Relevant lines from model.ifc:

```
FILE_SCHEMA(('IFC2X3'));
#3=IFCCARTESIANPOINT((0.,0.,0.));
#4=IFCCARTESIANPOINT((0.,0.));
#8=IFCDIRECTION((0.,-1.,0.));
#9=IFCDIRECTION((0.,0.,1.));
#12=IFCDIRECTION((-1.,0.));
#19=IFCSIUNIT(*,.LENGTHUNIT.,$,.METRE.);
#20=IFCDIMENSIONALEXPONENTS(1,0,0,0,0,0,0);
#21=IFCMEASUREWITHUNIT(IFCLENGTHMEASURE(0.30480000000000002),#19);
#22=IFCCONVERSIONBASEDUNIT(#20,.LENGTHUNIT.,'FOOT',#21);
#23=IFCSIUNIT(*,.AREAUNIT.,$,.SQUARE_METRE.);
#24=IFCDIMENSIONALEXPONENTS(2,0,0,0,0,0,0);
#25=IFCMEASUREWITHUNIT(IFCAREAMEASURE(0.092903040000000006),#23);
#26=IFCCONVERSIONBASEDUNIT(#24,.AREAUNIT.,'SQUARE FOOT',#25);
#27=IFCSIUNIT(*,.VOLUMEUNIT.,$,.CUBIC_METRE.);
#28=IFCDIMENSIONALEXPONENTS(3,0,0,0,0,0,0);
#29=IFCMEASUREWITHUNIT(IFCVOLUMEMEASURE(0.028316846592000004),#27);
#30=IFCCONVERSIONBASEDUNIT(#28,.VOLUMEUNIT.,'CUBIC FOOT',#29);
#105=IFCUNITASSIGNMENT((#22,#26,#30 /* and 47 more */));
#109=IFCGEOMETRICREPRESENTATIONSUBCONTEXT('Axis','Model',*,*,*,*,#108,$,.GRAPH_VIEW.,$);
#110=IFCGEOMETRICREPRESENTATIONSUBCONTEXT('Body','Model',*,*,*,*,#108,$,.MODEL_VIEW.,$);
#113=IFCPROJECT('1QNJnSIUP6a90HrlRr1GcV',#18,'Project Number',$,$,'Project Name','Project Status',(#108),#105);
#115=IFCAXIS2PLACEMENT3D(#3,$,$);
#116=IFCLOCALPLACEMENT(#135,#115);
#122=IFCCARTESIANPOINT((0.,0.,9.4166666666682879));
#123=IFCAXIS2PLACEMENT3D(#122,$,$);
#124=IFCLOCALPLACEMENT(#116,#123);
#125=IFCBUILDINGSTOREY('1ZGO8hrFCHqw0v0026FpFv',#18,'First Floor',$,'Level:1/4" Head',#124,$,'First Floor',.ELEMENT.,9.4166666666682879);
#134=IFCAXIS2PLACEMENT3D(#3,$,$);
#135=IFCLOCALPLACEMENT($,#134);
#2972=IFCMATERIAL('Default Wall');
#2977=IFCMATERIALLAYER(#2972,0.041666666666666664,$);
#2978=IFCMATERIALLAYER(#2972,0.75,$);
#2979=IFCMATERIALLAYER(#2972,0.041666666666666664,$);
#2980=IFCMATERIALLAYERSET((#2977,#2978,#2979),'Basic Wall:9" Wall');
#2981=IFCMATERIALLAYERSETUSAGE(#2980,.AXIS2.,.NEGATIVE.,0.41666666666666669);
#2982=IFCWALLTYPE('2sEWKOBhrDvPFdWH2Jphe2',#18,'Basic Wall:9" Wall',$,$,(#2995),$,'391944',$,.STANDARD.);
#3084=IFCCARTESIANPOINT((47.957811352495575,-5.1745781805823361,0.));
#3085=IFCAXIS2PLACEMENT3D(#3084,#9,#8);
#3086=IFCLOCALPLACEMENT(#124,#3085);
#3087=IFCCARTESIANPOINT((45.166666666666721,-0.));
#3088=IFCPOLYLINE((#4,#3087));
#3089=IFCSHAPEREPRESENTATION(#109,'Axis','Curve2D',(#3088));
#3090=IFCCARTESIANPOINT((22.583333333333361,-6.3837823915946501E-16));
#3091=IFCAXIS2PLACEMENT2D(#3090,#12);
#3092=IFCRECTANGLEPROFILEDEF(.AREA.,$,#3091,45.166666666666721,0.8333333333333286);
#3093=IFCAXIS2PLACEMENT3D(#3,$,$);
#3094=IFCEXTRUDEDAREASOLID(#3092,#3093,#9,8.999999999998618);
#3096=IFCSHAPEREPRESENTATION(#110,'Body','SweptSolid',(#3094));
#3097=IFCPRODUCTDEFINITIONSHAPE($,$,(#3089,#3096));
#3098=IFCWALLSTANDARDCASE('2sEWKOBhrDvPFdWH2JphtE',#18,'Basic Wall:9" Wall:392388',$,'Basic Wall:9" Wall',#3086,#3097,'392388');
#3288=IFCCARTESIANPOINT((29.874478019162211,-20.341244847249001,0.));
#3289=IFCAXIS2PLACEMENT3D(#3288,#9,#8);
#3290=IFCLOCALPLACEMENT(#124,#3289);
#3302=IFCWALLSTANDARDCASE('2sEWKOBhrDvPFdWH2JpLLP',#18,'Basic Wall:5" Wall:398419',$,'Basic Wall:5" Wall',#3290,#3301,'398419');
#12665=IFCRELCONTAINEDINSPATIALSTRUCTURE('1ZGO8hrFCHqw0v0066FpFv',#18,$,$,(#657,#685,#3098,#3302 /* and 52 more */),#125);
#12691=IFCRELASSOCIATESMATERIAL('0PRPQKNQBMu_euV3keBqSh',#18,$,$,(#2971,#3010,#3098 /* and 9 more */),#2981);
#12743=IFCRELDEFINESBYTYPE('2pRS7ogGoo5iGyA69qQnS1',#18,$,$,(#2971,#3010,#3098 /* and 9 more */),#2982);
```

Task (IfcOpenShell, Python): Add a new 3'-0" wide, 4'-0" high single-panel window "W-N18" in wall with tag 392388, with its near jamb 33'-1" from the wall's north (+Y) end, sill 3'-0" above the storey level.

```python
import numpy as np
import ifcopenshell
import ifcopenshell.api.feature
import ifcopenshell.api.geometry
import ifcopenshell.api.root
import ifcopenshell.api.spatial
import ifcopenshell.api.type
import ifcopenshell.geom
import ifcopenshell.util.element
import ifcopenshell.util.placement
import ifcopenshell.util.representation
import ifcopenshell.util.shape
import ifcopenshell.util.unit

model = ifcopenshell.open("model.ifc")
unit_scale = ifcopenshell.util.unit.calculate_unit_scale(model)
settings = ifcopenshell.geom.settings()


def volume(element):
    """Net volume in cubic metres, openings subtracted."""
    shape = ifcopenshell.geom.create_shape(settings, element)
    return ifcopenshell.util.shape.get_volume(shape.geometry)


wall = model.by_guid("2sEWKOBhrDvPFdWH2JphtE")
storey = ifcopenshell.util.element.get_container(wall, ifc_class="IfcBuildingStorey")
context = ifcopenshell.util.representation.get_context(model, "Model", "Body", "MODEL_VIEW")
before = volume(wall)

width, height, from_end, sill = 0.9144, 1.2192, 10.0838, 0.9144  # metres

# The wall runs along its own X axis, and the end named is its -X end.
wall_shape = ifcopenshell.geom.create_shape(settings, wall)
x, y, z = ifcopenshell.util.shape.get_vertices(wall_shape.geometry).T
start = x.min() + from_end
face, thickness = float(y.min()), float(y.max() - y.min())
wall_matrix = ifcopenshell.util.placement.get_local_placement(wall.ObjectPlacement)
level = ifcopenshell.util.placement.get_local_placement(storey.ObjectPlacement)[2, 3]


def in_wall(x, y):
    """Placement at x, y metres in the wall's axes, at sill height."""
    matrix = wall_matrix.copy()
    matrix[:, 3] = wall_matrix @ np.array([x / unit_scale, y / unit_scale, 0.0, 1.0])
    matrix[2, 3] = level + sill / unit_scale
    return matrix


# Opening: a box that overshoots both wall faces by 50 mm.
opening = ifcopenshell.api.root.create_entity(model, ifc_class="IfcOpeningElement")
box = ifcopenshell.api.geometry.add_wall_representation(
    model, context=context, length=width, height=height, thickness=thickness + 0.1
)
ifcopenshell.api.geometry.assign_representation(model, product=opening, representation=box)
ifcopenshell.api.geometry.edit_object_placement(model, product=opening, matrix=in_wall(start, face - 0.05), is_si=False)
ifcopenshell.api.feature.add_feature(model, feature=opening, element=wall)

window = ifcopenshell.api.root.create_entity(model, ifc_class="IfcWindow", name="W-N18")
window.OverallWidth, window.OverallHeight = width / unit_scale, height / unit_scale
body = ifcopenshell.api.geometry.add_window_representation(
    model,
    context=context,
    overall_width=window.OverallWidth,
    overall_height=window.OverallHeight,
    partition_type="SINGLE_PANEL",
)
ifcopenshell.api.geometry.assign_representation(model, product=window, representation=body)
ifcopenshell.api.spatial.assign_container(model, products=[window], relating_structure=storey)
fills = ifcopenshell.api.feature.add_filling(model, opening=opening, element=window)
fills.OwnerHistory = window.OwnerHistory  # required in IFC2X3

# IFC2X3 keeps the operation on the window style.
style = ifcopenshell.api.root.create_entity(model, ifc_class="IfcWindowStyle", name="W-N18")
style.OperationType, style.ConstructionType = "SINGLE_PANEL", "NOTDEFINED"
style.ParameterTakesPrecedence = style.Sizeable = False
ifcopenshell.api.type.assign_type(model, related_objects=[window], relating_type=style)

# Centre the window in the wall's thickness.
ifcopenshell.api.geometry.edit_object_placement(model, product=window, matrix=in_wall(start, face), is_si=False)
window_shape = ifcopenshell.geom.create_shape(settings, window)
depth = ifcopenshell.util.shape.get_vertices(window_shape.geometry)[:, 1]
offset = face + thickness / 2 - (depth.min() + depth.max()) / 2
ifcopenshell.api.geometry.edit_object_placement(model, product=window, matrix=in_wall(start, offset), is_si=False)

after = volume(wall)

print(f"wall volume {before:.3f} -> {after:.3f} m3")

model.write("model_v2.ifc")
```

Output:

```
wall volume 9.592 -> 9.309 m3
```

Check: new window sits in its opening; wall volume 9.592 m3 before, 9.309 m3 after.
